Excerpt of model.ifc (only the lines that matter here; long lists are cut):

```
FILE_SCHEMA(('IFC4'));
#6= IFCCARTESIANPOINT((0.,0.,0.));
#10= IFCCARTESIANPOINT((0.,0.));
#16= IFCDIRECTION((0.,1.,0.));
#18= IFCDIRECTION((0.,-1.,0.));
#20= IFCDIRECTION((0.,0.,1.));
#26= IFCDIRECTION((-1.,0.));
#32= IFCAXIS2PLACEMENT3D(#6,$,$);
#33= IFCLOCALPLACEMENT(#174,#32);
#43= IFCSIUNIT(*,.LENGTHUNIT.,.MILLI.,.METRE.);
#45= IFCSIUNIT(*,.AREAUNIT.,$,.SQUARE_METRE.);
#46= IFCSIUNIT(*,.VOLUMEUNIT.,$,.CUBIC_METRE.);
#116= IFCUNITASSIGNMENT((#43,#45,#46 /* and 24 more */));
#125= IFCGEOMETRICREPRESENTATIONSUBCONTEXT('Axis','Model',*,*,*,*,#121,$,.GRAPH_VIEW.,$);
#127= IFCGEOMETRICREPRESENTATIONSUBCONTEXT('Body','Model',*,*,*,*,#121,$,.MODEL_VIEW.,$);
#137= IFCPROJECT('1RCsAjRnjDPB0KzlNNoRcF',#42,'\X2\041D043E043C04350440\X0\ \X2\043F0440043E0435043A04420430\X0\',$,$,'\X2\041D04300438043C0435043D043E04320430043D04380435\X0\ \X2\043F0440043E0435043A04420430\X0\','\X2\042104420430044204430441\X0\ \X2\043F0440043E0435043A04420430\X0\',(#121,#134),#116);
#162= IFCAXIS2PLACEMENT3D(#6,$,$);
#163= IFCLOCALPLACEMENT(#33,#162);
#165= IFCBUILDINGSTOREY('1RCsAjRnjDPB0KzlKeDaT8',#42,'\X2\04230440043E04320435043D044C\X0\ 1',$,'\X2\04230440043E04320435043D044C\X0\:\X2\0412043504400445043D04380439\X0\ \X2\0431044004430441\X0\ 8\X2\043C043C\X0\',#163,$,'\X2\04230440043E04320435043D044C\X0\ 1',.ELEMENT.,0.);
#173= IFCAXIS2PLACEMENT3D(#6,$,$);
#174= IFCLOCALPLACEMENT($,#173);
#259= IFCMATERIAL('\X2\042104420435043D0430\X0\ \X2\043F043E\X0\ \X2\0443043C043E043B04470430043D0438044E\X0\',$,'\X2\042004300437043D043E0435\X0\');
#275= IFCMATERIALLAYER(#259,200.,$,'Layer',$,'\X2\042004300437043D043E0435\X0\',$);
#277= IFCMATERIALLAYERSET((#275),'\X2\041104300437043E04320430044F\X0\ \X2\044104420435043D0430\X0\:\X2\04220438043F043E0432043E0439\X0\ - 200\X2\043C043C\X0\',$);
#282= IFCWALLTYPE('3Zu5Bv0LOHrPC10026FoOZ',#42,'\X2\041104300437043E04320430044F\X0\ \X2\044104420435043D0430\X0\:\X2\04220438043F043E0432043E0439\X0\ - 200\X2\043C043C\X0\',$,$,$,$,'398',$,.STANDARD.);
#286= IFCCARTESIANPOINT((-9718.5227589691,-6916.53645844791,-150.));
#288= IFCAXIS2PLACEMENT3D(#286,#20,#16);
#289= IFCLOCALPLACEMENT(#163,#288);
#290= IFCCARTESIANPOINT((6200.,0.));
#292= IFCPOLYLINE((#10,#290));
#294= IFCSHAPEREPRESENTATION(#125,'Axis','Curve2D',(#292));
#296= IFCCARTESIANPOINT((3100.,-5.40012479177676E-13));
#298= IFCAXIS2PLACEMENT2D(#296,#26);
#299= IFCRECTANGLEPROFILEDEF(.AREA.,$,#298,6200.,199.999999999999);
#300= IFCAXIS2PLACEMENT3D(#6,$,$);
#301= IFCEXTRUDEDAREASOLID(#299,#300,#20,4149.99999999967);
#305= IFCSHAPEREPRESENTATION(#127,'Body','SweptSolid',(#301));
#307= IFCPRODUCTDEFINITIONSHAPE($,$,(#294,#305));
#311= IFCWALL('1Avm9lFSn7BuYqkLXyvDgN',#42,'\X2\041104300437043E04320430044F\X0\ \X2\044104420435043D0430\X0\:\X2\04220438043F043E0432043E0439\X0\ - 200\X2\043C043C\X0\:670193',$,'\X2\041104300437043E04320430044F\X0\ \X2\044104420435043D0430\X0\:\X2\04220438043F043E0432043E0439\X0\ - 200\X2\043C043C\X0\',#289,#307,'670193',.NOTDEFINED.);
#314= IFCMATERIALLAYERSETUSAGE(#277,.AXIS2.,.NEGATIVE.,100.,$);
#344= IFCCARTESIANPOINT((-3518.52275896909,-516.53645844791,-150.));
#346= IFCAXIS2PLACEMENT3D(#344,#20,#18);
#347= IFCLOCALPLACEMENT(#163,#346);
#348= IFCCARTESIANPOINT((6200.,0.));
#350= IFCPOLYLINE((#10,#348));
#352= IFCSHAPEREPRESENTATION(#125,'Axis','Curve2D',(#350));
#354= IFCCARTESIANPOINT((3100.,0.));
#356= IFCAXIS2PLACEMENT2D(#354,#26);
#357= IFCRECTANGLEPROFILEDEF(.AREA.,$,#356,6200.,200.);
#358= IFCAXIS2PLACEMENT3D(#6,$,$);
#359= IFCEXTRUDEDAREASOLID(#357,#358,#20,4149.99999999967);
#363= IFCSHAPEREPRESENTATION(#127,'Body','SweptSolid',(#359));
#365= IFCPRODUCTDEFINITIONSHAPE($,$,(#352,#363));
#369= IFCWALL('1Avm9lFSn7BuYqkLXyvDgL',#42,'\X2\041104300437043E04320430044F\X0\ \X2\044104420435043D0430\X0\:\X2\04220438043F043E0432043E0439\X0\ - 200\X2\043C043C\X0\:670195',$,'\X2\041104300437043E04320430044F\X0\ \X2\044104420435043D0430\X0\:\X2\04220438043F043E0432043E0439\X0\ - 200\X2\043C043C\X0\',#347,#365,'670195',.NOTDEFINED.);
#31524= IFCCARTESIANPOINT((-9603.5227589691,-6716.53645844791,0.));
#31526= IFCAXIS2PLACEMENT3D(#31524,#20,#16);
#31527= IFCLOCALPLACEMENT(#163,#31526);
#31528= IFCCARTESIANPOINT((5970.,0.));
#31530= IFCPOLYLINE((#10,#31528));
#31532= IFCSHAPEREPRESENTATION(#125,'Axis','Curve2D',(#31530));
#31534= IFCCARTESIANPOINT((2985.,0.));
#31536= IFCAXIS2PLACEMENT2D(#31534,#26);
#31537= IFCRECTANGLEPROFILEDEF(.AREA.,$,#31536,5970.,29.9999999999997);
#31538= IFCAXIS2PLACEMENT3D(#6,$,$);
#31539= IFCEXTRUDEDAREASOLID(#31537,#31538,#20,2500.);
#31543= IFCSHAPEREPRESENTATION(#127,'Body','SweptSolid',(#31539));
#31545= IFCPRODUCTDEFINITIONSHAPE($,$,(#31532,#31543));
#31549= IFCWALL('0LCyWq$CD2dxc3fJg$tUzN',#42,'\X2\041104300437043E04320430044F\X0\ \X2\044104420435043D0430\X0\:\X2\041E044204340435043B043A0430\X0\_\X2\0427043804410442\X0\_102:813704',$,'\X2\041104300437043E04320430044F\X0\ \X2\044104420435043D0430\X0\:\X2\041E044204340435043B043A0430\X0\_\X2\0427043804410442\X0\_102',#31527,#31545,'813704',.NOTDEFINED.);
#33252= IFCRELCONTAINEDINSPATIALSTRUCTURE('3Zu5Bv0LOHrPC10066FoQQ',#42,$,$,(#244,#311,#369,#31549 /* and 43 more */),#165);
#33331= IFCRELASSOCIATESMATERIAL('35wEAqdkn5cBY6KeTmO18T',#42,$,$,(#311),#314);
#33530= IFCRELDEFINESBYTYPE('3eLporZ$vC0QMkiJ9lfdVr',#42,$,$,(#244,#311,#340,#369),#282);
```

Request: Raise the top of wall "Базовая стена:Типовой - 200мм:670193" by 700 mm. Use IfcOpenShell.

```python
import ifcopenshell
import ifcopenshell.geom
import ifcopenshell.util.representation
import ifcopenshell.util.shape

model = ifcopenshell.open("model.ifc")
settings = ifcopenshell.geom.settings()


def volume(element):
    """Net volume in cubic metres, openings subtracted."""
    shape = ifcopenshell.geom.create_shape(settings, element)
    return ifcopenshell.util.shape.get_volume(shape.geometry)


wall = model.by_guid("1Avm9lFSn7BuYqkLXyvDgN")
before = volume(wall)

body = ifcopenshell.util.representation.get_representation(wall, "Model", "Body")
solid = body.Items[0]
old_height = solid.Depth
solid.Depth += 700.0
after = volume(wall)

print(f"height {old_height:g} -> {solid.Depth:g}, volume {before:.3f} -> {after:.3f} m3")

model.write("model_v2.ifc")
```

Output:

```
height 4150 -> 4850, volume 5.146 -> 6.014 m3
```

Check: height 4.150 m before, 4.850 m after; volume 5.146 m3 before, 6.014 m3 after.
